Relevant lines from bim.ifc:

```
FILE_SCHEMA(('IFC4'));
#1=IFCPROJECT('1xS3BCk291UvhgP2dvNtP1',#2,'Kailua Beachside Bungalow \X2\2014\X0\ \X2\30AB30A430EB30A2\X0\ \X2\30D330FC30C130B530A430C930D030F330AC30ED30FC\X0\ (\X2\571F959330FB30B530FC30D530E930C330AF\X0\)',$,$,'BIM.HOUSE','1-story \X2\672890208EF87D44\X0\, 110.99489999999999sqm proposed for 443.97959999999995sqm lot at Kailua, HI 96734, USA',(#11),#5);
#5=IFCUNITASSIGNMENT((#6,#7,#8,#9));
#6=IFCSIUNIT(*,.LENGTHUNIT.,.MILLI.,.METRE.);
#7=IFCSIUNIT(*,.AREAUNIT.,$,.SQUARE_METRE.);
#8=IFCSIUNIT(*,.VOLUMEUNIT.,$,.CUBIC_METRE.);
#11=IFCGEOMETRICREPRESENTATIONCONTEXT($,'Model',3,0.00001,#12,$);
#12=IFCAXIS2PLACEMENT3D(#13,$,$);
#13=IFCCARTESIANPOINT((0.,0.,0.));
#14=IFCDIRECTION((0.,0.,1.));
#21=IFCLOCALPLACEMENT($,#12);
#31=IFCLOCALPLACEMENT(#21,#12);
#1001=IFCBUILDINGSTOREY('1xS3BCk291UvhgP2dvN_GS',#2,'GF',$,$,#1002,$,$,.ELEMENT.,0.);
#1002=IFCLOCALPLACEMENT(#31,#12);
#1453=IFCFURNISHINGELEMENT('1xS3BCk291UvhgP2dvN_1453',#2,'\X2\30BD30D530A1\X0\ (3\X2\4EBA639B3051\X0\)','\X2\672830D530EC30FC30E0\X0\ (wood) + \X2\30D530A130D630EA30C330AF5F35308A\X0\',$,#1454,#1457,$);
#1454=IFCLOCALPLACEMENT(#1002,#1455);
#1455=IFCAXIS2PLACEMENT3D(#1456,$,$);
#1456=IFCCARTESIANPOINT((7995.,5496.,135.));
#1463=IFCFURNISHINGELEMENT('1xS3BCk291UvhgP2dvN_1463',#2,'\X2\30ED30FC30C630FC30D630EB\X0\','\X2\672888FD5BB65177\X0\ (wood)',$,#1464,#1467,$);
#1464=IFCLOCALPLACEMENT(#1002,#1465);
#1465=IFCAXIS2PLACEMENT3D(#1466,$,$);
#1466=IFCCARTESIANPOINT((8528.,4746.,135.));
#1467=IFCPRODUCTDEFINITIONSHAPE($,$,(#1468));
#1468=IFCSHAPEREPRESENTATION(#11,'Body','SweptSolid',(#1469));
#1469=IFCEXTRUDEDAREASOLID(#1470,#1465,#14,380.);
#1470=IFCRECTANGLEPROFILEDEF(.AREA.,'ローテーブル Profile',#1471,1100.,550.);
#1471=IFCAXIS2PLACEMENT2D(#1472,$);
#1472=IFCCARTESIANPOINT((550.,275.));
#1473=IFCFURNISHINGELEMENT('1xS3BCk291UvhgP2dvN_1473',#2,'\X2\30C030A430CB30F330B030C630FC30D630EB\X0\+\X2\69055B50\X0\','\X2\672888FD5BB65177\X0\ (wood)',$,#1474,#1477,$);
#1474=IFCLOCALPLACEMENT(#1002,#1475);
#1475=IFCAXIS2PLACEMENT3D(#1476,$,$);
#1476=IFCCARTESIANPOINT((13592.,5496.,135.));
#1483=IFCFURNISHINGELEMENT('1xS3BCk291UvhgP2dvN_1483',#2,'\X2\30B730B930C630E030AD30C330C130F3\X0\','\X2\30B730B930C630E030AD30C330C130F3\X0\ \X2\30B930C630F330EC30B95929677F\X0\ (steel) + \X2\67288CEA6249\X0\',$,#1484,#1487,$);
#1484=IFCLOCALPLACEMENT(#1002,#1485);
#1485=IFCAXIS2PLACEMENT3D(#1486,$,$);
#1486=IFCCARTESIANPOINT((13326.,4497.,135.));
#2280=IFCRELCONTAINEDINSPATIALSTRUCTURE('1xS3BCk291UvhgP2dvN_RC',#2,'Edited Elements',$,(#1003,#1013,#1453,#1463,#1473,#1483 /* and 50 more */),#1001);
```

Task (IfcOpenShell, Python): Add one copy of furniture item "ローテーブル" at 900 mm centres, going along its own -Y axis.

```python
import ifcopenshell
import ifcopenshell.api.geometry
import ifcopenshell.api.root
import ifcopenshell.util.element
import ifcopenshell.util.placement

model = ifcopenshell.open("bim.ifc")


def reuse_history(source, copy):
    """copy_class also copies each property set's owner history, people and application; keep the originals."""
    for rel in copy.IsDefinedBy:
        if rel.is_a("IfcRelDefinesByProperties") and (history := rel.RelatingPropertyDefinition.OwnerHistory):
            rel.RelatingPropertyDefinition.OwnerHistory = source.OwnerHistory
            ifcopenshell.util.element.remove_deep2(model, history)


source = model.by_guid("1xS3BCk291UvhgP2dvN_1463")
base = ifcopenshell.util.placement.get_local_placement(source.ObjectPlacement)
step = -base[:3, 1] * 900.0

for i in range(1, 2):
    copy = ifcopenshell.api.root.copy_class(model, product=source)
    copy.Representation = ifcopenshell.util.element.copy_deep(
        model, source.Representation, exclude=["IfcGeometricRepresentationContext", "IfcRepresentationMap"]
    )
    reuse_history(source, copy)
    matrix = base.copy()
    matrix[:3, 3] += i * step
    print("added at", matrix[:3, 3].round(3) + 0.0)
    ifcopenshell.api.geometry.edit_object_placement(model, product=copy, matrix=matrix, is_si=False)

model.write("bim_rev.ifc")
```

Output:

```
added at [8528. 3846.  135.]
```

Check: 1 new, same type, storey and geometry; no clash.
